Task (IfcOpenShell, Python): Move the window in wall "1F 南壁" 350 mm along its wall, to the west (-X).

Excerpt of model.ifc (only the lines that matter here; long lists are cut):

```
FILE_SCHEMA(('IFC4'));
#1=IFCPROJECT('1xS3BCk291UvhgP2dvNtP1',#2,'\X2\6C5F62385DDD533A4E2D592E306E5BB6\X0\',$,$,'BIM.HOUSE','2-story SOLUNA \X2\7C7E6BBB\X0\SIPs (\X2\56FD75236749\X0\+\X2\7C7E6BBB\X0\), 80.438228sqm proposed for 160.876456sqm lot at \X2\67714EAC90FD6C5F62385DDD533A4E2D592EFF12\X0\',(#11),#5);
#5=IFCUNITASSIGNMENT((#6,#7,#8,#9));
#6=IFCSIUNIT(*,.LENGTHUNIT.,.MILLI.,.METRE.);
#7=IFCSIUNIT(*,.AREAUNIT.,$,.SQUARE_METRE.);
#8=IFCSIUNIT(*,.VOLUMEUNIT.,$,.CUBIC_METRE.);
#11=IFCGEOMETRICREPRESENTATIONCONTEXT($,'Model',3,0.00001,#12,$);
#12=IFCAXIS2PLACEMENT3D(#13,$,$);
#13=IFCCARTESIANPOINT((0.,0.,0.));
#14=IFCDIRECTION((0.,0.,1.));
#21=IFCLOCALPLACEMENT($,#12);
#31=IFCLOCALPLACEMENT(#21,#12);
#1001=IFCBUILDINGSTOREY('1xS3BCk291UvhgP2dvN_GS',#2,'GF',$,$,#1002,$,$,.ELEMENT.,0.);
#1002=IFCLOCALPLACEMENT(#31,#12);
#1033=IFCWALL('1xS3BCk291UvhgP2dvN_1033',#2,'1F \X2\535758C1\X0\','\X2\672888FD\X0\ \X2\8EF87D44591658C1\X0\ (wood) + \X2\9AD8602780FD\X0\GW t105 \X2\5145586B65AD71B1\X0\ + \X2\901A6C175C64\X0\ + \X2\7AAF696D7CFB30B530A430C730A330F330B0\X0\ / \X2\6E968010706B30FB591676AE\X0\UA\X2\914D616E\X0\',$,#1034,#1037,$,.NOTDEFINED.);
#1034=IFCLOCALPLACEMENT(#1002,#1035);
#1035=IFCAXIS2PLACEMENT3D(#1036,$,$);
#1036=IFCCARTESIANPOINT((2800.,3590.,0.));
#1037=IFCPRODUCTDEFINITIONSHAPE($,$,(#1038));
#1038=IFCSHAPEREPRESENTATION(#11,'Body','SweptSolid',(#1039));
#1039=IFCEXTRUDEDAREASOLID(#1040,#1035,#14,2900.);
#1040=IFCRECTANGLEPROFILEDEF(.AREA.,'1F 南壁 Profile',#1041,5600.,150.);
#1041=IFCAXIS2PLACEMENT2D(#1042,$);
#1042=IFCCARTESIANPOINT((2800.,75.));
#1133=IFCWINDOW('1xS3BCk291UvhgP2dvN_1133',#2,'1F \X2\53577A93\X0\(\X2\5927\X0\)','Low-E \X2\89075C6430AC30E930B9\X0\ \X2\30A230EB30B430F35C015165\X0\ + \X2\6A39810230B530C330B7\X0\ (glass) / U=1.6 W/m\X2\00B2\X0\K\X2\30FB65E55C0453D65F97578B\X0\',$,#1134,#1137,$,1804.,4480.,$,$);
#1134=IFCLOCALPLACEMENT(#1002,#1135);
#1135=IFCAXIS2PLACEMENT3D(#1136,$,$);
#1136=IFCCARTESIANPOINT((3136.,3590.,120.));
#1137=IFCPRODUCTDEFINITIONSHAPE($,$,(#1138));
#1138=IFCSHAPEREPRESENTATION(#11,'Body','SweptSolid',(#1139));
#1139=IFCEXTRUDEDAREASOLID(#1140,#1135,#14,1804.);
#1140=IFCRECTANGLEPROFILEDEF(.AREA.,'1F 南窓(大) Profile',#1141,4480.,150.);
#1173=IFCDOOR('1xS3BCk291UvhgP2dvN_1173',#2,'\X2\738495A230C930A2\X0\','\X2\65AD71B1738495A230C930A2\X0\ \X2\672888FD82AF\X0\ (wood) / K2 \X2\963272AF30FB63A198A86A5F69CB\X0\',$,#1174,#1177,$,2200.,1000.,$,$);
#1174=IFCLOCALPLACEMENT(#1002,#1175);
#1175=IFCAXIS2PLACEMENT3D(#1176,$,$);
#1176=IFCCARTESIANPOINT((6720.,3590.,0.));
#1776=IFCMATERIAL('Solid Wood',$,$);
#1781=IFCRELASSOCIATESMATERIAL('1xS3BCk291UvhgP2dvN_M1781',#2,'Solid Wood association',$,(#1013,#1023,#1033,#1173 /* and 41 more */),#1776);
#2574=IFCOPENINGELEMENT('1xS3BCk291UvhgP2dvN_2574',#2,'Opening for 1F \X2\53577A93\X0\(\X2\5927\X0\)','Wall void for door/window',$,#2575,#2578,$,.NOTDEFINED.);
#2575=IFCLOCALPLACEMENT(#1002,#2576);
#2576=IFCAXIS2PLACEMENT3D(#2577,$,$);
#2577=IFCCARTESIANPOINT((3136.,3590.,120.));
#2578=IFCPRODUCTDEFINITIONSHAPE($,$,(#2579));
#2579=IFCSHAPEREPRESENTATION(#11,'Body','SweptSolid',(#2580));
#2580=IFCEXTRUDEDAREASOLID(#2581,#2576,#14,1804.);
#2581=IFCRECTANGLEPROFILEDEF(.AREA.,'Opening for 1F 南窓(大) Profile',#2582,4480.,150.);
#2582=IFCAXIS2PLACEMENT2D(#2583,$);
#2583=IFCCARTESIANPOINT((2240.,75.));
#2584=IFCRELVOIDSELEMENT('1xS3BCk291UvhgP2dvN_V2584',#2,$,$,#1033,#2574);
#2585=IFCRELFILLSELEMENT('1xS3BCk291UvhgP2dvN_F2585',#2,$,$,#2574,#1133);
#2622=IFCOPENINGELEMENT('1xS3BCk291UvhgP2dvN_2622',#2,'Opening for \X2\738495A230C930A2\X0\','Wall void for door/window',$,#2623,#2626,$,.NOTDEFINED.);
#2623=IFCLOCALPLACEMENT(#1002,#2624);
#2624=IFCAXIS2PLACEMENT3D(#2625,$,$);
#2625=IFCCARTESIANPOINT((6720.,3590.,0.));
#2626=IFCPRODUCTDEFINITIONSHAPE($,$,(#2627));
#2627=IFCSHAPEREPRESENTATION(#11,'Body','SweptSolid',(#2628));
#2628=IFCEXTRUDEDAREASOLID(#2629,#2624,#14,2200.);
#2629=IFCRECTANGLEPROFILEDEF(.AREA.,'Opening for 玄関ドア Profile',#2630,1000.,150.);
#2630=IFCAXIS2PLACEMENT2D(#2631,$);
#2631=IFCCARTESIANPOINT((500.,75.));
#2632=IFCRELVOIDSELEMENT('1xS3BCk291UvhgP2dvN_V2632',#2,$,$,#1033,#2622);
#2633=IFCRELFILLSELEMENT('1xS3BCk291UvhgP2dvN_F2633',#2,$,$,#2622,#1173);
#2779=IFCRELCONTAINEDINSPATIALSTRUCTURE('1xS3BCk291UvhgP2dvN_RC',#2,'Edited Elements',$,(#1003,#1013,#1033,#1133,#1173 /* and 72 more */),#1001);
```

```python
import ifcopenshell
import ifcopenshell.api.geometry
import ifcopenshell.util.placement

model = ifcopenshell.open("model.ifc")

window = model.by_guid("1xS3BCk291UvhgP2dvN_1133")
opening = window.FillsVoids[0].RelatingOpeningElement
wall = opening.VoidsElements[0].RelatingBuildingElement

wall_matrix = ifcopenshell.util.placement.get_local_placement(wall.ObjectPlacement)
shift = wall_matrix[:3, 0] * -350.0
before = ifcopenshell.util.placement.get_local_placement(window.ObjectPlacement)[:3, 3].copy()

# The window is not placed relative to its opening, so move both.
for product in (opening, window):
    matrix = ifcopenshell.util.placement.get_local_placement(product.ObjectPlacement)
    matrix[:3, 3] += shift
    ifcopenshell.api.geometry.edit_object_placement(model, product=product, matrix=matrix, is_si=False)

after = ifcopenshell.util.placement.get_local_placement(window.ObjectPlacement)[:3, 3]
print("window moved by", (after - before).round(3) + 0.0)

model.write("model_edited.ifc")
```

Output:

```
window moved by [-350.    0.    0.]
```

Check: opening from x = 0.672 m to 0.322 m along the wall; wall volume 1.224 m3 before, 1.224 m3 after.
